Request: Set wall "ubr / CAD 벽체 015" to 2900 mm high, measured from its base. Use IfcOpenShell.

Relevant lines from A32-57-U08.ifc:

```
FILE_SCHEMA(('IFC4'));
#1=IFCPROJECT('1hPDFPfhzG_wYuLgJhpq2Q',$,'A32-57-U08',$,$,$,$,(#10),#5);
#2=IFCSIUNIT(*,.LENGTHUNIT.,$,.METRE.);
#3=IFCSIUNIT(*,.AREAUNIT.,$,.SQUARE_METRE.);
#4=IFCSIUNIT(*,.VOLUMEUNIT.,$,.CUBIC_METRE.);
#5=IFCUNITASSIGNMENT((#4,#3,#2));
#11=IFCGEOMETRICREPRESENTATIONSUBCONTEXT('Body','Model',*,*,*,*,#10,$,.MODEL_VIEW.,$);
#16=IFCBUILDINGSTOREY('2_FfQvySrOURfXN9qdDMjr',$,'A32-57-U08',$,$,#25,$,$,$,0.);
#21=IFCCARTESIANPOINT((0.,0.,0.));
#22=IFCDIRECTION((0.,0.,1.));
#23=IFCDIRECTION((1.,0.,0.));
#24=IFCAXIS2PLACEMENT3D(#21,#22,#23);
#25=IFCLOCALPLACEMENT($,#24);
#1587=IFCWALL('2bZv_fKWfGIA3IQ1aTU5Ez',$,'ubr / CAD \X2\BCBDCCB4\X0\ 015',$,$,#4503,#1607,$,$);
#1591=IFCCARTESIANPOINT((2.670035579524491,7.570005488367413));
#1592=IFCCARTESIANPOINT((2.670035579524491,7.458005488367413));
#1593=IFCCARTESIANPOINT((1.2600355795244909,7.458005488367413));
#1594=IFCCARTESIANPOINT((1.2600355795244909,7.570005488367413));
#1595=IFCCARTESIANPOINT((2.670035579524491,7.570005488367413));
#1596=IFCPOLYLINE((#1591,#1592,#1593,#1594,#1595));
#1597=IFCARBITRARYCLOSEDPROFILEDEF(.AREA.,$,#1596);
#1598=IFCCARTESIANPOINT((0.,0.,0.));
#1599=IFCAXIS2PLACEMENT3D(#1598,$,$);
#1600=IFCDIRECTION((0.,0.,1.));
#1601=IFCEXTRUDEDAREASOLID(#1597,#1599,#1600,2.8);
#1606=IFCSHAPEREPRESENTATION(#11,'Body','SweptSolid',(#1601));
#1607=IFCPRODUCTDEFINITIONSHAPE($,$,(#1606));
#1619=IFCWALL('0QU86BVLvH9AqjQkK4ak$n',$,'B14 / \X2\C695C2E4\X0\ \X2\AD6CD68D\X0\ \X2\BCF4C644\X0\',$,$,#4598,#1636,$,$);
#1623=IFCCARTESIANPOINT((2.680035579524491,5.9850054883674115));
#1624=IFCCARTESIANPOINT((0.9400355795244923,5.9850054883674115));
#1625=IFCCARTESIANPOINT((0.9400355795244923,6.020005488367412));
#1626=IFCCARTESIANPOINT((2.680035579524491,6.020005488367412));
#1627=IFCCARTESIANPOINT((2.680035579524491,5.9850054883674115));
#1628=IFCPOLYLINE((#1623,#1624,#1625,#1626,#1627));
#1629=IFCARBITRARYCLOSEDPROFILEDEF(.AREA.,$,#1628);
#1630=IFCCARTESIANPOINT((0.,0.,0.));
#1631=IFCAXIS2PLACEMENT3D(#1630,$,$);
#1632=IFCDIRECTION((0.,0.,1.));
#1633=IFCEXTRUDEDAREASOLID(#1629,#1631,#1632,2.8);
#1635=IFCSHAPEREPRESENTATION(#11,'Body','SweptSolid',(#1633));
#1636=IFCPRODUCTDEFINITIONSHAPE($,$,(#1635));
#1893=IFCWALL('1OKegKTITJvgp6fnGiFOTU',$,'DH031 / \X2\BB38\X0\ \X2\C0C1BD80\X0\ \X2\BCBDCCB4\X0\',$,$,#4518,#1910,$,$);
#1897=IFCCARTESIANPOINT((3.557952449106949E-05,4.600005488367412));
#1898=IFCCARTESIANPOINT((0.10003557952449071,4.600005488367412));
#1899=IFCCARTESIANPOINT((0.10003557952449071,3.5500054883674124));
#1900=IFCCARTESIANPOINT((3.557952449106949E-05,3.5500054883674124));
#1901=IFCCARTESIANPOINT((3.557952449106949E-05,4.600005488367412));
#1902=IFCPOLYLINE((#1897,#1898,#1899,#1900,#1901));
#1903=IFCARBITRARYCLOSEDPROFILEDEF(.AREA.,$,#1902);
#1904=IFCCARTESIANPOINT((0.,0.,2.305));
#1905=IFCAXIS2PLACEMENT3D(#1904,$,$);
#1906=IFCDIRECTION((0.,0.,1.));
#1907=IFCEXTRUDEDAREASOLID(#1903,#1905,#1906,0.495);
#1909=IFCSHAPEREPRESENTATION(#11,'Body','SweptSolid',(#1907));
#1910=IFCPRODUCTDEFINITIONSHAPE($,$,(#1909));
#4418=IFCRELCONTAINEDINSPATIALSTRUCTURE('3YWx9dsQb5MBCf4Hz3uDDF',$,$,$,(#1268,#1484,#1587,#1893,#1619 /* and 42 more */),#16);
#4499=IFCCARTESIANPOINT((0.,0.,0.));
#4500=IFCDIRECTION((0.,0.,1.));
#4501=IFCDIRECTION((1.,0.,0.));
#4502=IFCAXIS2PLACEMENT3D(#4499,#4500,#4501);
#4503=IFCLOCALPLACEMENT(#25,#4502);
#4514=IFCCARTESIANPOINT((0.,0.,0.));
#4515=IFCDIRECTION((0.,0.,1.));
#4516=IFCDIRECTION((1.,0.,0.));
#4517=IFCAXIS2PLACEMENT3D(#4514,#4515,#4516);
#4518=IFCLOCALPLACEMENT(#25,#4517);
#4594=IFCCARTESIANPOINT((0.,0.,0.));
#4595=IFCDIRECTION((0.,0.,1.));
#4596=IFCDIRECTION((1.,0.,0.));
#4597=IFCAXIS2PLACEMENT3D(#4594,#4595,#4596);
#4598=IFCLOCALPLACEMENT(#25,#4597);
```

```python
import ifcopenshell
import ifcopenshell.geom
import ifcopenshell.util.representation
import ifcopenshell.util.shape

model = ifcopenshell.open("A32-57-U08.ifc")
settings = ifcopenshell.geom.settings()


def volume(element):
    """Net volume in cubic metres, openings subtracted."""
    shape = ifcopenshell.geom.create_shape(settings, element)
    return ifcopenshell.util.shape.get_volume(shape.geometry)


wall = model.by_guid("2bZv_fKWfGIA3IQ1aTU5Ez")
before = volume(wall)

body = ifcopenshell.util.representation.get_representation(wall, "Model", "Body")
solid = body.Items[0]
old_height = solid.Depth
solid.Depth = 2.9
after = volume(wall)

print(f"height {old_height:g} -> {solid.Depth:g}, volume {before:.3f} -> {after:.3f} m3")

model.write("A32-57-U08-out.ifc")
```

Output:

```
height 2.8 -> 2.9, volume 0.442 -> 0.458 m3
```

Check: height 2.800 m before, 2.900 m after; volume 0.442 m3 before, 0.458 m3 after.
